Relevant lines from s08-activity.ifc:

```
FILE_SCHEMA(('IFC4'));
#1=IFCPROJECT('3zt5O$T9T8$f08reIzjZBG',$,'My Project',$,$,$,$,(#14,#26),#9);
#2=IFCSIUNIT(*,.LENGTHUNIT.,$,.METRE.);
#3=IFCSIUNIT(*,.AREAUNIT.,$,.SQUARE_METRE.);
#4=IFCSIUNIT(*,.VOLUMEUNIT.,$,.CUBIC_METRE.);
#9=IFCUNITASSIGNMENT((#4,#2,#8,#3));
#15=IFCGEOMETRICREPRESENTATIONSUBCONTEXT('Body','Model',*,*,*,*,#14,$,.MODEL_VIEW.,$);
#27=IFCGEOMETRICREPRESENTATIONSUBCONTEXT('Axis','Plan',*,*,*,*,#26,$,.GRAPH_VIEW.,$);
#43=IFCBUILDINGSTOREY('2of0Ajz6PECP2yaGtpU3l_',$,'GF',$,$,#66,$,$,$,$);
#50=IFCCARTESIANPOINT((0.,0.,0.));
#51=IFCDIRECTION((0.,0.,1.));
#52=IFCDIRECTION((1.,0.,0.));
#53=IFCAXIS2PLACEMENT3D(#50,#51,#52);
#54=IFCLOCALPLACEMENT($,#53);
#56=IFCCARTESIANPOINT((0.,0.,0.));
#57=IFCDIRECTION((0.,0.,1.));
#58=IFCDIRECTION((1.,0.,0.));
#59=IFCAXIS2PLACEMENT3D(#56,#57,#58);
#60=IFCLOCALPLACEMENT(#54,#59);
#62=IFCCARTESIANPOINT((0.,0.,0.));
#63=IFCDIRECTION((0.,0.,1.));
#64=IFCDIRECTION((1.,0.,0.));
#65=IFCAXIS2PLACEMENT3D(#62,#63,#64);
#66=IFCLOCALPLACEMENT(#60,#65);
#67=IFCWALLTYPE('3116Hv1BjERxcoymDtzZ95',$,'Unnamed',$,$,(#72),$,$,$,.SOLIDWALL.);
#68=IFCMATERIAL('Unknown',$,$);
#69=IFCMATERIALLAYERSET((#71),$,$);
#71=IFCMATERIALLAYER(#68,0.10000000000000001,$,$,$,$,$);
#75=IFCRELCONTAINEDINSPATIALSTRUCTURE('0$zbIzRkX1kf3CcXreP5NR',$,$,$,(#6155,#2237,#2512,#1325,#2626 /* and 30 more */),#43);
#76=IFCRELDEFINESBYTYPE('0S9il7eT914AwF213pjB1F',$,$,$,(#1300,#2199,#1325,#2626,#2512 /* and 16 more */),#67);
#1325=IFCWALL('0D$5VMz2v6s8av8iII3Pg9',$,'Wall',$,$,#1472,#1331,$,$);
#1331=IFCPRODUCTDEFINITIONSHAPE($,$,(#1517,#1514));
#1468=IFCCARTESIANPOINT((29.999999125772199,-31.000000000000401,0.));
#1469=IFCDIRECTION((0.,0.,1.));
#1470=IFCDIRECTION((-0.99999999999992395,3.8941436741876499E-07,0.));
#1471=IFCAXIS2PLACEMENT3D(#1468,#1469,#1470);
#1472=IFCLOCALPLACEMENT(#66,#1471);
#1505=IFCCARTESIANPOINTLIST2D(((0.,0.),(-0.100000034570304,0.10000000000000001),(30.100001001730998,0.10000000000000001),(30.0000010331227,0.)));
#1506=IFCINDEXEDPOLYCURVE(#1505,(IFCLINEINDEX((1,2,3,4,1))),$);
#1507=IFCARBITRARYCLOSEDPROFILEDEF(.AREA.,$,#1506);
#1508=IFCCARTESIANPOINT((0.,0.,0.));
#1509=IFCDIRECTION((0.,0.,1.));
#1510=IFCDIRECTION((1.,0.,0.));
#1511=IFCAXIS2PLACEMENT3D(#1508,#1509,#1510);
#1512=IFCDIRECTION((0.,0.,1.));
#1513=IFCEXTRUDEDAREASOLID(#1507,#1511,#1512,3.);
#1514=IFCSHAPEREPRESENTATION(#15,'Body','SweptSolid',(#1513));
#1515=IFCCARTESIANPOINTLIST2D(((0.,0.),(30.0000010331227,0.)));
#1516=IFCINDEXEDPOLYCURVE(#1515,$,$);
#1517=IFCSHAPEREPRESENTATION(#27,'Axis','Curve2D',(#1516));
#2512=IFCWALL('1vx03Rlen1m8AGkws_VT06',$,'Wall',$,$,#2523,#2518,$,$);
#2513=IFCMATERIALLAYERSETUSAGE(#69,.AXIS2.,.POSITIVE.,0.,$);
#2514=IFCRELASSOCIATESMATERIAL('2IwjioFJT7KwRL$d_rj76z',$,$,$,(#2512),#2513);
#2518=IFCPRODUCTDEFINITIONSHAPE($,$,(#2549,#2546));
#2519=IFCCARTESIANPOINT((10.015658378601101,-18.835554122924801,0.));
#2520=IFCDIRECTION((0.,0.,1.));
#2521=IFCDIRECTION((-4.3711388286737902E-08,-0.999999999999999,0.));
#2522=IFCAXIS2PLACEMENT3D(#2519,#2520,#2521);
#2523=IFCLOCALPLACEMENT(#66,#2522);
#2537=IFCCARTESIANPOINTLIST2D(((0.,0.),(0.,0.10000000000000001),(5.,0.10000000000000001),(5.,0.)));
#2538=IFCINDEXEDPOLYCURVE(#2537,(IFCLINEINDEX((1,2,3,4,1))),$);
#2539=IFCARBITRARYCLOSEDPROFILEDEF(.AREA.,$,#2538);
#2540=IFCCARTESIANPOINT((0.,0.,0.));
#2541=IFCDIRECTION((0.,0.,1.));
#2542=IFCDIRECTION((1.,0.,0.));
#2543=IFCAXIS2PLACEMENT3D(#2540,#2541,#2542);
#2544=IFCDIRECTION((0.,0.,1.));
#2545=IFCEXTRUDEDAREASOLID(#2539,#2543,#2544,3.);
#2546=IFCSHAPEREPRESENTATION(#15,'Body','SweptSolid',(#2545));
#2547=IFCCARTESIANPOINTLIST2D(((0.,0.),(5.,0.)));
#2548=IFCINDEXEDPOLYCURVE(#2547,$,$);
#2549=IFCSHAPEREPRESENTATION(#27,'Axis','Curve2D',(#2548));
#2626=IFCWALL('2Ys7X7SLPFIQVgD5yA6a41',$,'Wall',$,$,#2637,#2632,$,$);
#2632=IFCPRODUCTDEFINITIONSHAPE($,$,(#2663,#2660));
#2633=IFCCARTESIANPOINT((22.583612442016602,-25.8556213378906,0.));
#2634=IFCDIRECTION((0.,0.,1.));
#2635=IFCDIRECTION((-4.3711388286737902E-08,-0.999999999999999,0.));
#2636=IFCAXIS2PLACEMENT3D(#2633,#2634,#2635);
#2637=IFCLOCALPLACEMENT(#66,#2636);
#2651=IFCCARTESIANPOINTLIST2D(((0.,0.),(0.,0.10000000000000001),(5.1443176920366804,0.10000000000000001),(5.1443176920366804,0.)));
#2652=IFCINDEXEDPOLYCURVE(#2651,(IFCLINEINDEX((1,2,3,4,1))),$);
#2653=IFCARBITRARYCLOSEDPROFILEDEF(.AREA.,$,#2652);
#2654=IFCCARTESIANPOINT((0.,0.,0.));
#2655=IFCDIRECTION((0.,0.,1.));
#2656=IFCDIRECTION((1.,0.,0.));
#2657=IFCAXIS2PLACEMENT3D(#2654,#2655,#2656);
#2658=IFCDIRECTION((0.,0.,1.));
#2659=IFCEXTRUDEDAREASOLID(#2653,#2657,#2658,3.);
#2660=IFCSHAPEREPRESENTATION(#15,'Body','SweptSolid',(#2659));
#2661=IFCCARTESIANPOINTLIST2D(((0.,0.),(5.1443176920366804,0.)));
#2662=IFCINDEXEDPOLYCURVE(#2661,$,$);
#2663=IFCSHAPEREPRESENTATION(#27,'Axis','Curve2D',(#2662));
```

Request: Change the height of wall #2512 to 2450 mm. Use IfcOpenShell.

```python
import ifcopenshell
import ifcopenshell.geom
import ifcopenshell.util.representation
import ifcopenshell.util.shape
import ifcopenshell.util.unit

model = ifcopenshell.open("s08-activity.ifc")
unit_scale = ifcopenshell.util.unit.calculate_unit_scale(model)
settings = ifcopenshell.geom.settings()


def volume(element):
    """Net volume in cubic metres, openings subtracted."""
    shape = ifcopenshell.geom.create_shape(settings, element)
    return ifcopenshell.util.shape.get_volume(shape.geometry)


wall = model.by_guid("1vx03Rlen1m8AGkws_VT06")
before = volume(wall)

body = ifcopenshell.util.representation.get_representation(wall, "Model", "Body")
solid = body.Items[0]
old_height = solid.Depth
solid.Depth = 2.45 / unit_scale
after = volume(wall)

print(f"height {old_height:g} -> {solid.Depth:g}, volume {before:.3f} -> {after:.3f} m3")

model.write("s08-activity_rev.ifc")
```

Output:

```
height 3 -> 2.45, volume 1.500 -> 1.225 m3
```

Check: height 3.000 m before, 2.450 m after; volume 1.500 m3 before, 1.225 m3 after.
